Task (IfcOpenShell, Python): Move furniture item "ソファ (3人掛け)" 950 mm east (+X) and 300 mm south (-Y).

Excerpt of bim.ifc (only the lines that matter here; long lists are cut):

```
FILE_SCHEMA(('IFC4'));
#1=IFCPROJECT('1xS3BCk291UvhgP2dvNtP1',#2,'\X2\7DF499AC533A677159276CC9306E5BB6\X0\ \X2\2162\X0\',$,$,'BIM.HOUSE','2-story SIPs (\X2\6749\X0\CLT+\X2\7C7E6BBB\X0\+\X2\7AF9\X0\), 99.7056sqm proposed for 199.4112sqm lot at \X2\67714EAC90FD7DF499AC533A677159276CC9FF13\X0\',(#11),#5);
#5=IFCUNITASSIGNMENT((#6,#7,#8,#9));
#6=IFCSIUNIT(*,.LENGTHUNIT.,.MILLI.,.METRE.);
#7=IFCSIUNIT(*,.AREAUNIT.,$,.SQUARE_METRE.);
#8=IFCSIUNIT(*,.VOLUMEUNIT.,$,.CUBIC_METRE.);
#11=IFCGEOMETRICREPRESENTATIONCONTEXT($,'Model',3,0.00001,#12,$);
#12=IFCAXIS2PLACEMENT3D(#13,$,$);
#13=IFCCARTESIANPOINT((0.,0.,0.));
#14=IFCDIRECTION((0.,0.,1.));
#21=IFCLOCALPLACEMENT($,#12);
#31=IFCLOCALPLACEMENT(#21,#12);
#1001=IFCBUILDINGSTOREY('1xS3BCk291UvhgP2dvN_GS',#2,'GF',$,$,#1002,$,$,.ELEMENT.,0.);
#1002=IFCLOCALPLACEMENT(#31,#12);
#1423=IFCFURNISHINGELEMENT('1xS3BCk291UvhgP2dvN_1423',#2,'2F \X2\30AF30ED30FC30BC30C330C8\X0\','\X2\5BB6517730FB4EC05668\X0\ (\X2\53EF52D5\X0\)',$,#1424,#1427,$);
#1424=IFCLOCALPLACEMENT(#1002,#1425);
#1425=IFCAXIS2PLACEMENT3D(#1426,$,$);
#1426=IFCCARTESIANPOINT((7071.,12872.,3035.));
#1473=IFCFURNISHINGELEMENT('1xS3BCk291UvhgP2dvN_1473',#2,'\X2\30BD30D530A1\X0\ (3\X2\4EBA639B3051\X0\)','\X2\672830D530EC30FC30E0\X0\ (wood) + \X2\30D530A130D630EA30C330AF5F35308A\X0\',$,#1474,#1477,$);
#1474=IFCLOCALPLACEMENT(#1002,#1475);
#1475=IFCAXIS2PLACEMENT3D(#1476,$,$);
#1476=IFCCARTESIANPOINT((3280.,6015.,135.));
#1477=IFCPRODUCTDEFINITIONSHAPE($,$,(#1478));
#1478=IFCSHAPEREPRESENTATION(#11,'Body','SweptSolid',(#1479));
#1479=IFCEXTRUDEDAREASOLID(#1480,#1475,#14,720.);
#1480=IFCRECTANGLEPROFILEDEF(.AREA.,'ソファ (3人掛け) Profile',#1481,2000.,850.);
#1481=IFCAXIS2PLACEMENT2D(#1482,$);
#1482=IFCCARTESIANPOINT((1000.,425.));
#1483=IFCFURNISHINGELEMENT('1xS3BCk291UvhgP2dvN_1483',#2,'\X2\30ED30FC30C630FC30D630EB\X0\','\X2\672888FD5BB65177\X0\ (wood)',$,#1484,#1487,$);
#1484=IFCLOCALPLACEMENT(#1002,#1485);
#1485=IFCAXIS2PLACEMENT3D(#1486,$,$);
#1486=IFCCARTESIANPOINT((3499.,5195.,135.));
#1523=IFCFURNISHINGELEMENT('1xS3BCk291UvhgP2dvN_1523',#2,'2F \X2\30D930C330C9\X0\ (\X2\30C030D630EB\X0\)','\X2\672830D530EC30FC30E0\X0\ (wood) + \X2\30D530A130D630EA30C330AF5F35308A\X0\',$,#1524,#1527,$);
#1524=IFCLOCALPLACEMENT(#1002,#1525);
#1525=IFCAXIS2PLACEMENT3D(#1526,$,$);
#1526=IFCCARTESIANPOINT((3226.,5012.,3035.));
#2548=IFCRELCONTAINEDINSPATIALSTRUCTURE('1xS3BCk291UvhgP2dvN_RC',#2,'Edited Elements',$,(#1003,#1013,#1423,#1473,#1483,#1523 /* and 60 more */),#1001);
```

```python
import ifcopenshell
import ifcopenshell.api.geometry
import ifcopenshell.util.placement

model = ifcopenshell.open("bim.ifc")

item = model.by_guid("1xS3BCk291UvhgP2dvN_1473")
matrix = ifcopenshell.util.placement.get_local_placement(item.ObjectPlacement)
matrix[0, 3] += 950.0
matrix[1, 3] -= 300.0
ifcopenshell.api.geometry.edit_object_placement(model, product=item, matrix=matrix, is_si=False)

print(ifcopenshell.util.placement.get_local_placement(item.ObjectPlacement).round(3) + 0.0)

model.write("bim_rev.ifc")
```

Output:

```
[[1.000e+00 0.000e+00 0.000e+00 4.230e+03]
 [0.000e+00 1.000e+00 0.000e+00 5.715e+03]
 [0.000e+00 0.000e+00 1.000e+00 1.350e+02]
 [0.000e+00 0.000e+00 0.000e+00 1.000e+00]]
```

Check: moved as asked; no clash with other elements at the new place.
